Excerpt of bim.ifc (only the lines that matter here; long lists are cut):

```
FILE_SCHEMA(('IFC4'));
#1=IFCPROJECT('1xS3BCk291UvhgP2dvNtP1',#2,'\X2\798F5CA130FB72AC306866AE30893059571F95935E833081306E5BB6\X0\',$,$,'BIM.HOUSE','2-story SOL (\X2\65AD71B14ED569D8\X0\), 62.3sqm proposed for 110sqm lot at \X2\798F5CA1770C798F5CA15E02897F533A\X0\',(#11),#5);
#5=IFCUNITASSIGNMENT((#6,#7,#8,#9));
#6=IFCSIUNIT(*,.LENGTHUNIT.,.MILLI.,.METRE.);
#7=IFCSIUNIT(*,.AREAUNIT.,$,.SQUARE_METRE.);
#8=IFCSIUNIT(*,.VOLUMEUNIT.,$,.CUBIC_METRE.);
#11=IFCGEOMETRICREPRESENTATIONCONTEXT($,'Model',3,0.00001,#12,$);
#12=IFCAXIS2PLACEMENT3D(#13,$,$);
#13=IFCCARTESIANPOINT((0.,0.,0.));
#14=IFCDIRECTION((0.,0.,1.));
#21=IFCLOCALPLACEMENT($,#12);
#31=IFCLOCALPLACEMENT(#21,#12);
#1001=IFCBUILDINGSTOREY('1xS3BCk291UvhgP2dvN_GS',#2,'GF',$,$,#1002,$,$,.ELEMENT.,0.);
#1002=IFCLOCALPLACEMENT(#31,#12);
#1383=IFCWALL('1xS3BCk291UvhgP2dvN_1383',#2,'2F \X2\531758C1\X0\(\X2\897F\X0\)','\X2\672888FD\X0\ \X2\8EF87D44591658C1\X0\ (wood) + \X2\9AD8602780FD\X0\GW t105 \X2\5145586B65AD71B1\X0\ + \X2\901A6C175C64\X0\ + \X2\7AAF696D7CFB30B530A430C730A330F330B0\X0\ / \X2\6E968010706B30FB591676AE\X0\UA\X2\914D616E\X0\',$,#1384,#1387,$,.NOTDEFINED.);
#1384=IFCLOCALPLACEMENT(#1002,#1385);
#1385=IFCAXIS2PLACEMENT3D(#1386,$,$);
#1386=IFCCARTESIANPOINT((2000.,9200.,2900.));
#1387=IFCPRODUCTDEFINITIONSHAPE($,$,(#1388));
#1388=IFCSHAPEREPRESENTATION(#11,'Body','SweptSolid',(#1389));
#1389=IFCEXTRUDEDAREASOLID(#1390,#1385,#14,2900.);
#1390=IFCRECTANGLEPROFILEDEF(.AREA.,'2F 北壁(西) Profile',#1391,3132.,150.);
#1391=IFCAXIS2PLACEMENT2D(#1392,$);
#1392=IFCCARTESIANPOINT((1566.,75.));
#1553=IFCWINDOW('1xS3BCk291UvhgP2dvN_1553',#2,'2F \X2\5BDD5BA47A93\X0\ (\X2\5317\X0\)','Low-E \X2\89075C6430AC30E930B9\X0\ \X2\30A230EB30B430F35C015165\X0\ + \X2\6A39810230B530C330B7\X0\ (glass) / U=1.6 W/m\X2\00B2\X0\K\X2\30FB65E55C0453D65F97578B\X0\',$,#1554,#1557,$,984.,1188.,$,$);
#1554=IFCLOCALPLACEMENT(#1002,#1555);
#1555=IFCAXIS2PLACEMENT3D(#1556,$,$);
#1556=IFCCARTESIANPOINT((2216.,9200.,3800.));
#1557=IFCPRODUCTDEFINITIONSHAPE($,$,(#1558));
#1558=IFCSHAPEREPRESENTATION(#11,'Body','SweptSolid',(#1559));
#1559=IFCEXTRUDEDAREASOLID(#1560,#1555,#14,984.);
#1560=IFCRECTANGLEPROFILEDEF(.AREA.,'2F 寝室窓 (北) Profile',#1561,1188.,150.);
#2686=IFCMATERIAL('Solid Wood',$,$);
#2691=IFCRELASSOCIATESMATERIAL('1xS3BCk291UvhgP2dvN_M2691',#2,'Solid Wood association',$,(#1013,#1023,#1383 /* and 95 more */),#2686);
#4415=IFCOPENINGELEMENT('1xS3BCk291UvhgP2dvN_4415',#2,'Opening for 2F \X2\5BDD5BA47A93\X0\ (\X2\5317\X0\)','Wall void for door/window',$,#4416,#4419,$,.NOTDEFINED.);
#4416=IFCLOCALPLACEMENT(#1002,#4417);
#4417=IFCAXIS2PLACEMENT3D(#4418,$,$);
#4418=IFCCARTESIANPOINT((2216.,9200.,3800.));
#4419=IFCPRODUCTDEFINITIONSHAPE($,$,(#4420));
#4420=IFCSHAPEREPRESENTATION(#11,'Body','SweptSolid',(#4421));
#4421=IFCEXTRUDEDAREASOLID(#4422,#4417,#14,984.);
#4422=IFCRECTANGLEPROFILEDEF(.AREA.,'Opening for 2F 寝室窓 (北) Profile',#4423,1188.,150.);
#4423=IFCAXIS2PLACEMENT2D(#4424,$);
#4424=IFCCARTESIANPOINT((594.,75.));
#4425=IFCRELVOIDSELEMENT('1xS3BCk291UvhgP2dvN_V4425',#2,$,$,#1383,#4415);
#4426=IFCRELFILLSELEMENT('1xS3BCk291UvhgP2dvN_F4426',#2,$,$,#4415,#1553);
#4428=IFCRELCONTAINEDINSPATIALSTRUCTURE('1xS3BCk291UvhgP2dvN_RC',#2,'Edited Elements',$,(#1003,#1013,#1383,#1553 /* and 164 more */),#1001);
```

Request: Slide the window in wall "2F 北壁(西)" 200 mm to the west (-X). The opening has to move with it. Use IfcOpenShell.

```python
import ifcopenshell
import ifcopenshell.api.geometry
import ifcopenshell.util.placement
import ifcopenshell.util.unit

model = ifcopenshell.open("bim.ifc")
unit_scale = ifcopenshell.util.unit.calculate_unit_scale(model)

window = model.by_guid("1xS3BCk291UvhgP2dvN_1553")
opening = window.FillsVoids[0].RelatingOpeningElement
wall = opening.VoidsElements[0].RelatingBuildingElement

wall_matrix = ifcopenshell.util.placement.get_local_placement(wall.ObjectPlacement)
shift = wall_matrix[:3, 0] * -0.2 / unit_scale
before = ifcopenshell.util.placement.get_local_placement(window.ObjectPlacement)[:3, 3].copy()

# The window is not placed relative to its opening, so move both.
for product in (opening, window):
    matrix = ifcopenshell.util.placement.get_local_placement(product.ObjectPlacement)
    matrix[:3, 3] += shift
    ifcopenshell.api.geometry.edit_object_placement(model, product=product, matrix=matrix, is_si=False)

after = ifcopenshell.util.placement.get_local_placement(window.ObjectPlacement)[:3, 3]
print("window moved by", (after - before).round(3) + 0.0)

model.write("bim_updated.ifc")
```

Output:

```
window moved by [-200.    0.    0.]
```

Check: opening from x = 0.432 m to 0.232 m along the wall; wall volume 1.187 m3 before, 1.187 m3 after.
